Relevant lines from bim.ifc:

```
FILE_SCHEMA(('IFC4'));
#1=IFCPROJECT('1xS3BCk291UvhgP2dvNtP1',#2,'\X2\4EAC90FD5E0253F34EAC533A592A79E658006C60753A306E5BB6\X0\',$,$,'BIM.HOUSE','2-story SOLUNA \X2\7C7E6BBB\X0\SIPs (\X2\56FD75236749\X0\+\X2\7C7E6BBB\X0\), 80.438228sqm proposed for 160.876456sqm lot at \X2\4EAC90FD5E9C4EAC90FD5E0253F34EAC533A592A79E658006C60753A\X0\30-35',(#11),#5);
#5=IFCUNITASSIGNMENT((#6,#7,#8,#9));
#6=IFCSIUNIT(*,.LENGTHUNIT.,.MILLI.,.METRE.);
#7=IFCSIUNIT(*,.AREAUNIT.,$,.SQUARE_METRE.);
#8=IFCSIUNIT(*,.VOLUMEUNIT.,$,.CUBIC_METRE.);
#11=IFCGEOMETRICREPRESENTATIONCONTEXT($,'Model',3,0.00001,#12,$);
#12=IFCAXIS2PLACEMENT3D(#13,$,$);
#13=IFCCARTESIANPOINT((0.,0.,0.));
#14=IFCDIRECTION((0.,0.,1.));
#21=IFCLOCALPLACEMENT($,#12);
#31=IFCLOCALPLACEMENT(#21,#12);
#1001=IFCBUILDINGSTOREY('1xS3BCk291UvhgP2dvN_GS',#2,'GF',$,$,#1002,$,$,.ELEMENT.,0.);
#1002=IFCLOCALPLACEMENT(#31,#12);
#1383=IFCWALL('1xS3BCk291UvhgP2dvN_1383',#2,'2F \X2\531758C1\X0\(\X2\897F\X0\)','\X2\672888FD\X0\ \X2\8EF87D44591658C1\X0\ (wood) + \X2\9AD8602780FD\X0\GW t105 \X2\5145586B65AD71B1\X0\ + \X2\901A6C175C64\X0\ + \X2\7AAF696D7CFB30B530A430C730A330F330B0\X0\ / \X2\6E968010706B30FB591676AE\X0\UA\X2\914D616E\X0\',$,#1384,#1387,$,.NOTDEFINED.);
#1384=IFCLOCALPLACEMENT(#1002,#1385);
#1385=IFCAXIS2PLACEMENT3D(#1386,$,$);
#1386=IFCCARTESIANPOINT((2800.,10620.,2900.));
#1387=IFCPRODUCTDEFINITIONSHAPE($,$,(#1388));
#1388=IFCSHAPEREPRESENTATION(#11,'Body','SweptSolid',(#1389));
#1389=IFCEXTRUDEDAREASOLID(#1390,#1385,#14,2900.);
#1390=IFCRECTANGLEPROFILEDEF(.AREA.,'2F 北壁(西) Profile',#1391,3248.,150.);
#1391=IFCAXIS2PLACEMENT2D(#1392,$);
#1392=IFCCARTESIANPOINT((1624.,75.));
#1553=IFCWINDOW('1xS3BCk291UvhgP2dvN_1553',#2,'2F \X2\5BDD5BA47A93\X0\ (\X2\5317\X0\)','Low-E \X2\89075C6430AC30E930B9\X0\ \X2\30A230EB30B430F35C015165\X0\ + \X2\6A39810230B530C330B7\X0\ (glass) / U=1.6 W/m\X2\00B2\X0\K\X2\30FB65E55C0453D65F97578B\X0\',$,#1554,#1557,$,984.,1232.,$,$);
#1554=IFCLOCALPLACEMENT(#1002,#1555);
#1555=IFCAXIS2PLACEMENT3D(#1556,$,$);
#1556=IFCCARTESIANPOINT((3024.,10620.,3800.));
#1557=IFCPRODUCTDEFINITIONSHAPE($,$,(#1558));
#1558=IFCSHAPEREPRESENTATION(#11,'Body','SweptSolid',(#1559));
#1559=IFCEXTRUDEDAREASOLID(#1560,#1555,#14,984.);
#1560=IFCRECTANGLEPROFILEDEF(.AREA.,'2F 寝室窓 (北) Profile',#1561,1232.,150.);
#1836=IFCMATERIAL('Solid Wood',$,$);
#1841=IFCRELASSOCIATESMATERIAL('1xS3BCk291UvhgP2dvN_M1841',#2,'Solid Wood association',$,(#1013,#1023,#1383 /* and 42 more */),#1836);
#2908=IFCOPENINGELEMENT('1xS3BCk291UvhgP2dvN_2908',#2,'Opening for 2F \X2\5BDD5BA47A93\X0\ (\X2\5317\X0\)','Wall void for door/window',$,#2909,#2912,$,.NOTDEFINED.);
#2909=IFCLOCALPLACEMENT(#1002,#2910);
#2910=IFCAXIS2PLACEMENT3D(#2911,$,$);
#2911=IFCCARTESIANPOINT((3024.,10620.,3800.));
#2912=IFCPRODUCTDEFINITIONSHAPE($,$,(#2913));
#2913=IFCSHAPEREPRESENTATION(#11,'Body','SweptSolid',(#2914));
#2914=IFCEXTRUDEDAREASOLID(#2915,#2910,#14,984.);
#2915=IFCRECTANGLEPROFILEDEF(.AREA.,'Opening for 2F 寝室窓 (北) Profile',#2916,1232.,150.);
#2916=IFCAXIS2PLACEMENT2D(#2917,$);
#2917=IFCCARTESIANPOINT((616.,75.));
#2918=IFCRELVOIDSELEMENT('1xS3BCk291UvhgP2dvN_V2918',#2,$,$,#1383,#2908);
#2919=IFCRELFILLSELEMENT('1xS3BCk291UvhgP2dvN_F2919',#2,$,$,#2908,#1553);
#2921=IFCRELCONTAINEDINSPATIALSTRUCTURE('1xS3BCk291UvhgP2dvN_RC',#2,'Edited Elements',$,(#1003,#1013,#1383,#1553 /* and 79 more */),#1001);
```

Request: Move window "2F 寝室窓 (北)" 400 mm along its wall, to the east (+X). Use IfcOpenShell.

```python
import ifcopenshell
import ifcopenshell.api.geometry
import ifcopenshell.util.placement

model = ifcopenshell.open("bim.ifc")

window = model.by_guid("1xS3BCk291UvhgP2dvN_1553")
opening = window.FillsVoids[0].RelatingOpeningElement
wall = opening.VoidsElements[0].RelatingBuildingElement

wall_matrix = ifcopenshell.util.placement.get_local_placement(wall.ObjectPlacement)
shift = wall_matrix[:3, 0] * 400.0
before = ifcopenshell.util.placement.get_local_placement(window.ObjectPlacement)[:3, 3].copy()

# The window is not placed relative to its opening, so move both.
for product in (opening, window):
    matrix = ifcopenshell.util.placement.get_local_placement(product.ObjectPlacement)
    matrix[:3, 3] += shift
    ifcopenshell.api.geometry.edit_object_placement(model, product=product, matrix=matrix, is_si=False)

after = ifcopenshell.util.placement.get_local_placement(window.ObjectPlacement)[:3, 3]
print("window moved by", (after - before).round(3) + 0.0)

model.write("bim_edited.ifc")
```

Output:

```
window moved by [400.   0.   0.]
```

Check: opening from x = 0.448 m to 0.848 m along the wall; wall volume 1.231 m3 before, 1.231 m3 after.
